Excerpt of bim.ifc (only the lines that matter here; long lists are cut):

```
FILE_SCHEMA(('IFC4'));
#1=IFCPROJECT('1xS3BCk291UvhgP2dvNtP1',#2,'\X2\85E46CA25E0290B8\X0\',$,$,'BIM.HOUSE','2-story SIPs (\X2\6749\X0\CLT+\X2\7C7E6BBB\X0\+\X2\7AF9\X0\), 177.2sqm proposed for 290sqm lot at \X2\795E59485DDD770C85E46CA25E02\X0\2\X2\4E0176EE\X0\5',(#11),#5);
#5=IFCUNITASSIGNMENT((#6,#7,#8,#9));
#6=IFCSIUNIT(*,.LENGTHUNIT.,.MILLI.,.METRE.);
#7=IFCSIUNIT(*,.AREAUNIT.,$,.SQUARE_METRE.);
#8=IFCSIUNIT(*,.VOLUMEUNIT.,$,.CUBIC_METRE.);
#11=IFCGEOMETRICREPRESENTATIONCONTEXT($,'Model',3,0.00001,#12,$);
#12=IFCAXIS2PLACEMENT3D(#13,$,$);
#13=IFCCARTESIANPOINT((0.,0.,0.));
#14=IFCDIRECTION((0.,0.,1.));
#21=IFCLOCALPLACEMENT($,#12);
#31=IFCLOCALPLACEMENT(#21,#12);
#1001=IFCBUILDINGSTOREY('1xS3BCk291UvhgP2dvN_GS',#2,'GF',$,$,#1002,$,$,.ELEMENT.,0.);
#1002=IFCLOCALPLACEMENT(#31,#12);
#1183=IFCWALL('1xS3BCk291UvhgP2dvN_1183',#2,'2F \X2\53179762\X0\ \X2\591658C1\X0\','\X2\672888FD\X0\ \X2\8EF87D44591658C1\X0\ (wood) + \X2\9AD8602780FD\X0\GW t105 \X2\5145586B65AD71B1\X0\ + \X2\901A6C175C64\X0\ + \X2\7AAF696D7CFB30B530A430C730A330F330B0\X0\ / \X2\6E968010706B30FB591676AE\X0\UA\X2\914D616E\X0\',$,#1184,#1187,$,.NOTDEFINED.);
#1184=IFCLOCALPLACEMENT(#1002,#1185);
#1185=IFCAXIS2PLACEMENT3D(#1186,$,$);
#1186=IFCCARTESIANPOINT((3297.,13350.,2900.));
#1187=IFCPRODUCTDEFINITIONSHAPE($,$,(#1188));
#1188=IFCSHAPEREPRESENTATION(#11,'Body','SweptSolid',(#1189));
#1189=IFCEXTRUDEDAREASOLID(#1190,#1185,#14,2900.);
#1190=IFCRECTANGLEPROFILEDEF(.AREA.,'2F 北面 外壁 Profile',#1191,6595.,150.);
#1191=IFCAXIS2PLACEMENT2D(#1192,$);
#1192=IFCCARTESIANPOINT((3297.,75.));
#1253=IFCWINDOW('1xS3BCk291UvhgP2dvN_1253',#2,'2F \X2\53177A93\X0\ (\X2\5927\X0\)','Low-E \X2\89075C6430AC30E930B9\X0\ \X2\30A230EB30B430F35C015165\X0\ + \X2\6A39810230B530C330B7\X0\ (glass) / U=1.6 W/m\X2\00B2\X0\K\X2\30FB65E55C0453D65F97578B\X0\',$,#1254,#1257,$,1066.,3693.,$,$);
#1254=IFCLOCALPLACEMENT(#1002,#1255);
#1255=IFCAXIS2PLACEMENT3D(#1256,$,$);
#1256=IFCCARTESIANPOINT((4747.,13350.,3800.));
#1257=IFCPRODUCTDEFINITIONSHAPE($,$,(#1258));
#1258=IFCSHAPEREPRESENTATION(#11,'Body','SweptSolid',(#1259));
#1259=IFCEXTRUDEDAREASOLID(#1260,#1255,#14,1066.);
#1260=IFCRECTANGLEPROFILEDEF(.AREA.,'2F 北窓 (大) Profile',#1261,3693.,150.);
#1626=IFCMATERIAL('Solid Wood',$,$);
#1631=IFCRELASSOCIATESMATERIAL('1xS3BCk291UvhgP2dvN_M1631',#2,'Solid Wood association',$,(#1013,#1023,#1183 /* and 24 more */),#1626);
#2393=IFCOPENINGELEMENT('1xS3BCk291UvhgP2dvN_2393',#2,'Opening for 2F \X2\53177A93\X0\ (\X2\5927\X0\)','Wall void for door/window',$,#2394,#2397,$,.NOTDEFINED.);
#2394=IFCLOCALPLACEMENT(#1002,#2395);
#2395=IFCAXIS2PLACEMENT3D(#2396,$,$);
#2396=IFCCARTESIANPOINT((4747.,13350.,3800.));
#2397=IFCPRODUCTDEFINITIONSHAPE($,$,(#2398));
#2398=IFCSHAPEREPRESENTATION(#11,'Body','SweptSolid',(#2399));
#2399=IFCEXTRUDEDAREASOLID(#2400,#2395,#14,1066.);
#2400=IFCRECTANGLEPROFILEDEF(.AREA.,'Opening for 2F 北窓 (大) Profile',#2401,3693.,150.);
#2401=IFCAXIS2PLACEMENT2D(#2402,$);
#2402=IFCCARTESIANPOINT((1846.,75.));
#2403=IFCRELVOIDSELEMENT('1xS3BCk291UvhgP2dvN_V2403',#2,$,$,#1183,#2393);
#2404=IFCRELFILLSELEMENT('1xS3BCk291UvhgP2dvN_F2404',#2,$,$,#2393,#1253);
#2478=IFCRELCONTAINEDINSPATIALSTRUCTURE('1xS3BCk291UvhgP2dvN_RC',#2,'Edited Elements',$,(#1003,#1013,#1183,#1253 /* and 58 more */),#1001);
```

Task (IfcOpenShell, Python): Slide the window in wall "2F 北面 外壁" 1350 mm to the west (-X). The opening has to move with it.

```python
import ifcopenshell
import ifcopenshell.api.geometry
import ifcopenshell.util.placement
import ifcopenshell.util.unit

model = ifcopenshell.open("bim.ifc")
unit_scale = ifcopenshell.util.unit.calculate_unit_scale(model)

window = model.by_guid("1xS3BCk291UvhgP2dvN_1253")
opening = window.FillsVoids[0].RelatingOpeningElement
wall = opening.VoidsElements[0].RelatingBuildingElement

wall_matrix = ifcopenshell.util.placement.get_local_placement(wall.ObjectPlacement)
shift = wall_matrix[:3, 0] * -1.35 / unit_scale
before = ifcopenshell.util.placement.get_local_placement(window.ObjectPlacement)[:3, 3].copy()

# The window is not placed relative to its opening, so move both.
for product in (opening, window):
    matrix = ifcopenshell.util.placement.get_local_placement(product.ObjectPlacement)
    matrix[:3, 3] += shift
    ifcopenshell.api.geometry.edit_object_placement(model, product=product, matrix=matrix, is_si=False)

after = ifcopenshell.util.placement.get_local_placement(window.ObjectPlacement)[:3, 3]
print("window moved by", (after - before).round(3) + 0.0)

model.write("bim_edited.ifc")
```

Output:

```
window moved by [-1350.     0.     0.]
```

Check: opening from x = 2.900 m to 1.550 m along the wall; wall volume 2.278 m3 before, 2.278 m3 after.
